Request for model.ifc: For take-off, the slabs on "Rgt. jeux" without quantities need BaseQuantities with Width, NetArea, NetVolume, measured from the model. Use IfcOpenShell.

First a look at what the model holds.

```python
import ifcopenshell
import ifcopenshell.util.element
import ifcopenshell.util.unit

model = ifcopenshell.open("model.ifc")
print(model.schema)
for unit_type in ("LENGTHUNIT", "AREAUNIT", "VOLUMEUNIT"):
    print(unit_type, ifcopenshell.util.unit.calculate_unit_scale(model, unit_type))
storey = next(s for s in model.by_type("IfcBuildingStorey") if s.Name == "Rgt. jeux")
slabs = [e for e in ifcopenshell.util.element.get_decomposition(storey) if e.is_a("IfcSlab")]
for e in sorted(slabs, key=lambda e: e.id()):
    print(e.id(), e.is_a(), e.Name, list(ifcopenshell.util.element.get_psets(e, qtos_only=True)), sep=" | ")
```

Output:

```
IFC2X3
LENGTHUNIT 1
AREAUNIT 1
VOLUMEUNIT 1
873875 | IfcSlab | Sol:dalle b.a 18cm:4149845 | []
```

```python
import ifcopenshell
import ifcopenshell.api.pset
import ifcopenshell.geom
import ifcopenshell.util.element
import ifcopenshell.util.shape
import ifcopenshell.util.unit

model = ifcopenshell.open("model.ifc")
unit_scale = ifcopenshell.util.unit.calculate_unit_scale(model)
area_scale = ifcopenshell.util.unit.calculate_unit_scale(model, "AREAUNIT")
volume_scale = ifcopenshell.util.unit.calculate_unit_scale(model, "VOLUMEUNIT")
settings = ifcopenshell.geom.settings()

storey = next(s for s in model.by_type("IfcBuildingStorey") if s.Name == "Rgt. jeux")
slabs = [e for e in ifcopenshell.util.element.get_decomposition(storey) if e.is_a("IfcSlab")]

for e in sorted(slabs, key=lambda e: e.id()):
    if ifcopenshell.util.element.get_psets(e, qtos_only=True, should_inherit=False):
        continue
    # Geometry comes back in metres, in the element's own axes.
    shape = ifcopenshell.geom.create_shape(settings, e)
    values = {
        "Width": ifcopenshell.util.shape.get_z(shape.geometry) / unit_scale,
        "NetArea": ifcopenshell.util.shape.get_footprint_area(shape.geometry) / area_scale,
        "NetVolume": ifcopenshell.util.shape.get_volume(shape.geometry) / volume_scale,
    }
    qto = ifcopenshell.api.pset.add_qto(model, product=e, name="BaseQuantities")
    ifcopenshell.api.pset.edit_qto(model, qto=qto, properties=values)
    print(e.id(), {k: round(v, 3) for k, v in values.items()})

model.write("model_updated.ifc")
```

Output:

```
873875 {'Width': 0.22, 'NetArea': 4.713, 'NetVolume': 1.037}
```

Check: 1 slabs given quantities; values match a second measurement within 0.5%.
